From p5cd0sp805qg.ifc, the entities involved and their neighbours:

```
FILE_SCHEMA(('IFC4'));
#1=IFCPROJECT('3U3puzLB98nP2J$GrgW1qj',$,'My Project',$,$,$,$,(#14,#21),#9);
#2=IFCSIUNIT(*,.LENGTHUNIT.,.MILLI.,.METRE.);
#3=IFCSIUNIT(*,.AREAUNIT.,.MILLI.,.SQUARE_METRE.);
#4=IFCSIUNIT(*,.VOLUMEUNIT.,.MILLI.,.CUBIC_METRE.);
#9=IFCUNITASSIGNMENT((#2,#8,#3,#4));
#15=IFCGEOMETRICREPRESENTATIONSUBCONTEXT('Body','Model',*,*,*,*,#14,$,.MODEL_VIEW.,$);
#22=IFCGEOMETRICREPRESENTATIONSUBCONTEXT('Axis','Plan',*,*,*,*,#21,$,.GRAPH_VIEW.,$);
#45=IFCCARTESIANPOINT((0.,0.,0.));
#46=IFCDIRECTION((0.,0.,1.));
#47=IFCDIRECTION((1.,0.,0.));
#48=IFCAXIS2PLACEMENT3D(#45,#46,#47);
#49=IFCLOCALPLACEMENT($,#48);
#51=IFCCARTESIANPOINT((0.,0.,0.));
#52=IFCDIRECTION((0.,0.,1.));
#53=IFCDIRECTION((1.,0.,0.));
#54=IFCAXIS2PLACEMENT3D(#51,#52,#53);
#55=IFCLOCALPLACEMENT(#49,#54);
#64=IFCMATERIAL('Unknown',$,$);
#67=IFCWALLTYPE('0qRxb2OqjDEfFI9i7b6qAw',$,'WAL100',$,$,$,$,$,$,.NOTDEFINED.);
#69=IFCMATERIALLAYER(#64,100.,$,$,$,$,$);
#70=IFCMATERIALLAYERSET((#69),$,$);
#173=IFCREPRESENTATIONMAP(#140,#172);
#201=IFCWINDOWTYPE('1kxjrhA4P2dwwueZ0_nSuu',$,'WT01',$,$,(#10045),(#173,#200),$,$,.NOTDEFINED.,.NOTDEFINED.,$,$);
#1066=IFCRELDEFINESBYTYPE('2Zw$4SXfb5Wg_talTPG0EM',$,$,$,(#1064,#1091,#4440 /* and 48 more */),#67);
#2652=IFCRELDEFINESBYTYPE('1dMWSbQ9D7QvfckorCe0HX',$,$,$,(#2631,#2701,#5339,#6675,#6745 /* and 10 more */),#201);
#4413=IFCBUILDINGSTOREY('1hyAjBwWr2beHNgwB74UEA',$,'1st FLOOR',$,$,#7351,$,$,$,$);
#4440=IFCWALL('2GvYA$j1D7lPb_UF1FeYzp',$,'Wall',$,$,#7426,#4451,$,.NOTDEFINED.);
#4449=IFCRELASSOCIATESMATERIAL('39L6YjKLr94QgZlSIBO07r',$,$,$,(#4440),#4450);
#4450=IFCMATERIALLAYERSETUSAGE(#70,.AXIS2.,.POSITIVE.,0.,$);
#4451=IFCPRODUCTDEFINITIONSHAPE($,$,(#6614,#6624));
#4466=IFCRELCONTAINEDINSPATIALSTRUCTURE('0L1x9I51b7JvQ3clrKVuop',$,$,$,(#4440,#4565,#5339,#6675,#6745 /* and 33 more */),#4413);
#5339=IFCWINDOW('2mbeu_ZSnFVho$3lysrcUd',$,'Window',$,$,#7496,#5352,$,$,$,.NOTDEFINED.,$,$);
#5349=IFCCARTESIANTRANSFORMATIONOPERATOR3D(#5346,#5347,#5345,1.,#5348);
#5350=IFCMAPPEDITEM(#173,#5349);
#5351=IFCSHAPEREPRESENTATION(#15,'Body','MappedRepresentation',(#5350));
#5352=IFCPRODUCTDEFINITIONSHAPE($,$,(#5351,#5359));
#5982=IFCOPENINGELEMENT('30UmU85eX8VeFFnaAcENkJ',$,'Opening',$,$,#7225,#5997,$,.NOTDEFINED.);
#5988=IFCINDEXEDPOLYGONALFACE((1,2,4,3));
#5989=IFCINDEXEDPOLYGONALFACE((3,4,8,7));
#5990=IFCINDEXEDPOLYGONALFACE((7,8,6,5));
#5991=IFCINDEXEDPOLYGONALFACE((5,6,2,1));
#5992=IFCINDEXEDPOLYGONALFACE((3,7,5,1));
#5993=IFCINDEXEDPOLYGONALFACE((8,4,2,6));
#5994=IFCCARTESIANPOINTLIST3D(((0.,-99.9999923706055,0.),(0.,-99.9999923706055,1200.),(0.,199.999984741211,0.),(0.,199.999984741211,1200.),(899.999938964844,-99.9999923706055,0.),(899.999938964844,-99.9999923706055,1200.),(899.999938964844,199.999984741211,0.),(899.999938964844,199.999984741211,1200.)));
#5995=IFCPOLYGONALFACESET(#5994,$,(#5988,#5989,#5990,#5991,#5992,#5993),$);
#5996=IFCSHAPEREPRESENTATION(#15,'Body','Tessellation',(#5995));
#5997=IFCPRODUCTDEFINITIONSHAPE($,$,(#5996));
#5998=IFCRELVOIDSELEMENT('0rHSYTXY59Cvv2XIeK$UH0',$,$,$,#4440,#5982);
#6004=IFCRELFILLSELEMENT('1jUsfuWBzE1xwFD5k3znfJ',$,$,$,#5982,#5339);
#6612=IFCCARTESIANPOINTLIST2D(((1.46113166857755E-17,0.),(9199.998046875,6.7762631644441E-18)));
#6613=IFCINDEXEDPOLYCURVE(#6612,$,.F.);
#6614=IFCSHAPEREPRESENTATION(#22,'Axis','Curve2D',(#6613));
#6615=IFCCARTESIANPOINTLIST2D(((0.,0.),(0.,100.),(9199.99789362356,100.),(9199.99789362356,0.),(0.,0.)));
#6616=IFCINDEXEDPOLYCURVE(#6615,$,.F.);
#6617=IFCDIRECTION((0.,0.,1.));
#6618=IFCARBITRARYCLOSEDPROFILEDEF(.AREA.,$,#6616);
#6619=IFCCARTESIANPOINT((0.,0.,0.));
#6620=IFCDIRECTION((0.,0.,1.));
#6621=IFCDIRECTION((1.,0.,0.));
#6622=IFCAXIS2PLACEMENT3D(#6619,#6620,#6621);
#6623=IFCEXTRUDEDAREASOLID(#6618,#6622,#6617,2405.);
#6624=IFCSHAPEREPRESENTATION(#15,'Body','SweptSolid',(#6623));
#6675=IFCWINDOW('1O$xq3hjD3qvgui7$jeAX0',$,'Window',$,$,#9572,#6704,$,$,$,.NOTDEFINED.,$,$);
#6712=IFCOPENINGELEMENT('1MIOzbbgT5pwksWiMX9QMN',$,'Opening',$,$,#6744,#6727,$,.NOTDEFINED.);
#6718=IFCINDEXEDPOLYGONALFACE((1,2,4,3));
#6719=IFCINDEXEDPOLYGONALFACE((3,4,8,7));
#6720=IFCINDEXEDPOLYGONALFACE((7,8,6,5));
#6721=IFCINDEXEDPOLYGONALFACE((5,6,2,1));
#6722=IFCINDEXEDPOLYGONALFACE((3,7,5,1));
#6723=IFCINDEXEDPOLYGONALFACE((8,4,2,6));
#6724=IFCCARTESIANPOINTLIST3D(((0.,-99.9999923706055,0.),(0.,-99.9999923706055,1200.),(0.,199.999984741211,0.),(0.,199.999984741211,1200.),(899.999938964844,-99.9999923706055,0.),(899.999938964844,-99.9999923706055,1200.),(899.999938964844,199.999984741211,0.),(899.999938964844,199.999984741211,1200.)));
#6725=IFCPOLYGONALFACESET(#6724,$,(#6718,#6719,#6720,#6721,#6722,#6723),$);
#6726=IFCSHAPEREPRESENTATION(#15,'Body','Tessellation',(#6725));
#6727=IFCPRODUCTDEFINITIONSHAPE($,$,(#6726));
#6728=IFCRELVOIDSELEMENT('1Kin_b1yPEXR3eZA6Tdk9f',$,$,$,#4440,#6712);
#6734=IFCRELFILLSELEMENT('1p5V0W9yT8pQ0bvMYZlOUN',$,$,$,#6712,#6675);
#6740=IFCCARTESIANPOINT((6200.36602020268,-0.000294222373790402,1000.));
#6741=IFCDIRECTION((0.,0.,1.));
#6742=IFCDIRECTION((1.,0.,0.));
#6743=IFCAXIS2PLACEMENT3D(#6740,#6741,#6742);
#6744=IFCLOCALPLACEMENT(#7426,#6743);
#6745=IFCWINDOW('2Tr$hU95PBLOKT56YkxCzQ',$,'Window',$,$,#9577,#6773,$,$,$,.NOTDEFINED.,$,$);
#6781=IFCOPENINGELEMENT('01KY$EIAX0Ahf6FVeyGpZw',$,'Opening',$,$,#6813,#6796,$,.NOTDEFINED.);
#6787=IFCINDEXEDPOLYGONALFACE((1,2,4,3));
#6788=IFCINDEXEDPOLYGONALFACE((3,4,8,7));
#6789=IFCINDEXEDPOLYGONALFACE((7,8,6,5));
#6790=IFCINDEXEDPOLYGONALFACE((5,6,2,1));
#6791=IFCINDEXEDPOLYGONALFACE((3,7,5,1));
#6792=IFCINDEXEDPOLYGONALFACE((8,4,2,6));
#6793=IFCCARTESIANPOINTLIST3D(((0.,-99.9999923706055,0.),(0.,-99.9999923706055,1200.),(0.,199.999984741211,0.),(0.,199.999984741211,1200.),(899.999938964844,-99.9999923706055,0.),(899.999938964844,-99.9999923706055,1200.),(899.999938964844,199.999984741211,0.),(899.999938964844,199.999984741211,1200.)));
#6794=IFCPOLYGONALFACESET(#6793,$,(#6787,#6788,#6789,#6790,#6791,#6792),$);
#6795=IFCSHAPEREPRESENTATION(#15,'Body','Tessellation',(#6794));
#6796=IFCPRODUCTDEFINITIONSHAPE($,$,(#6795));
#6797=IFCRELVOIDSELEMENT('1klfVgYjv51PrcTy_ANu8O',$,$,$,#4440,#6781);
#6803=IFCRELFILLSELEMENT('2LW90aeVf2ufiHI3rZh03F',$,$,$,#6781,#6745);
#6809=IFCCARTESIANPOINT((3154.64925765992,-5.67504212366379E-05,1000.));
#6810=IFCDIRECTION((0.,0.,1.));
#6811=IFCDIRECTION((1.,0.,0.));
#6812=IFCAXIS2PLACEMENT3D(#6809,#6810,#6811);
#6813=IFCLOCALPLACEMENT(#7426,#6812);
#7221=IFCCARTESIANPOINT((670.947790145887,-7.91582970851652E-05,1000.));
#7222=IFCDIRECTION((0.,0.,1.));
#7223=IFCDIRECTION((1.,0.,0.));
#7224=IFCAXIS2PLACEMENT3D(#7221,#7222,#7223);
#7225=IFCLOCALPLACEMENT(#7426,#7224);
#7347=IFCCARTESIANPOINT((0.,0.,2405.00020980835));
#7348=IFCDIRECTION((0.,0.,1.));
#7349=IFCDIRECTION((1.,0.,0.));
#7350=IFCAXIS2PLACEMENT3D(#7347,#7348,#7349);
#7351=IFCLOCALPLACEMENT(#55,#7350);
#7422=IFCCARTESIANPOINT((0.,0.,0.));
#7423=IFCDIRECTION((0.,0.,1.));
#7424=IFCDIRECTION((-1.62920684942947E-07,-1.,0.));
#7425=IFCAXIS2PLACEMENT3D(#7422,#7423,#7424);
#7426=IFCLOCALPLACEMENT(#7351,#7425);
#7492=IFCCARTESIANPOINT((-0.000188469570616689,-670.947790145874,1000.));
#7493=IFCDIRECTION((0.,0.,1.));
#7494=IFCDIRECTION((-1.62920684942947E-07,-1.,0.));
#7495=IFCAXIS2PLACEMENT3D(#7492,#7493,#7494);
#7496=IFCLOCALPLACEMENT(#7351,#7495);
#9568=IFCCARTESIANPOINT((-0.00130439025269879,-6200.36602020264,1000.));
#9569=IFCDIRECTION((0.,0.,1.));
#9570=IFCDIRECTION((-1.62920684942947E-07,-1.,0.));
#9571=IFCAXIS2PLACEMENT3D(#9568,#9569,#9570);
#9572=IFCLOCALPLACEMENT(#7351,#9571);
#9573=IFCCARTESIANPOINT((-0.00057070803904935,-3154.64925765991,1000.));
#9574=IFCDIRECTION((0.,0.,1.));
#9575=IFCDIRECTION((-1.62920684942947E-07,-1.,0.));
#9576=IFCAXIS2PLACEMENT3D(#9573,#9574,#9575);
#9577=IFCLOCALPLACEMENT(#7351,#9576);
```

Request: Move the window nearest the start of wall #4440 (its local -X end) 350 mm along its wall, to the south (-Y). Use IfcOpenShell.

```python
import ifcopenshell
import ifcopenshell.api.geometry
import ifcopenshell.util.placement

model = ifcopenshell.open("p5cd0sp805qg.ifc")

window = model.by_guid("2mbeu_ZSnFVho$3lysrcUd")
opening = window.FillsVoids[0].RelatingOpeningElement
wall = opening.VoidsElements[0].RelatingBuildingElement

wall_matrix = ifcopenshell.util.placement.get_local_placement(wall.ObjectPlacement)
shift = wall_matrix[:3, 0] * 350.0
before = ifcopenshell.util.placement.get_local_placement(window.ObjectPlacement)[:3, 3].copy()

# The window is not placed relative to its opening, so move both.
for product in (opening, window):
    matrix = ifcopenshell.util.placement.get_local_placement(product.ObjectPlacement)
    matrix[:3, 3] += shift
    ifcopenshell.api.geometry.edit_object_placement(model, product=product, matrix=matrix, is_si=False)

after = ifcopenshell.util.placement.get_local_placement(window.ObjectPlacement)[:3, 3]
print("window moved by", (after - before).round(3) + 0.0)

model.write("p5cd0sp805qg_v2.ifc")
```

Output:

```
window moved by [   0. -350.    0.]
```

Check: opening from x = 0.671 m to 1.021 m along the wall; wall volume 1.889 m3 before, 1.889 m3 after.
